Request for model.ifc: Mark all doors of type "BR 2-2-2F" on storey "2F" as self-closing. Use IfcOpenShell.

First a look at what the model holds.

```python
import ifcopenshell
import ifcopenshell.util.element

model = ifcopenshell.open("model.ifc")
print(model.schema)
storey = next(s for s in model.by_type("IfcBuildingStorey") if s.Name == "2F")
doors = [e for e in ifcopenshell.util.element.get_decomposition(storey) if e.is_a("IfcDoor")]
seen = {}
for e in doors:
    element_type = ifcopenshell.util.element.get_type(e)
    key = (element_type.Name if element_type != e and element_type else None, ifcopenshell.util.element.get_pset(e, "Pset_DoorCommon", "SelfClosing"))
    seen[key] = seen.get(key, 0) + 1
for (name, value), count in sorted(seen.items(), key=str):
    print(count, "x", name, "|", value)
```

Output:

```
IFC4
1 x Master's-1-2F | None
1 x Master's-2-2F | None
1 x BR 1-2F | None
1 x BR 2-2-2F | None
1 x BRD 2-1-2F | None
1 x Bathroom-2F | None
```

```python
import ifcopenshell
import ifcopenshell.api.pset
import ifcopenshell.util.element

model = ifcopenshell.open("model.ifc")

storey = next(s for s in model.by_type("IfcBuildingStorey") if s.Name == "2F")
doors = [e for e in ifcopenshell.util.element.get_decomposition(storey) if e.is_a("IfcDoor")]

count = 0
for e in doors:
    element_type = ifcopenshell.util.element.get_type(e)
    if element_type in (None, e) or element_type.Name != "BR 2-2-2F":
        continue
    # add_pset returns the element's existing set when there is one.
    pset = ifcopenshell.api.pset.add_pset(model, product=e, name="Pset_DoorCommon")
    ifcopenshell.api.pset.edit_pset(model, pset=pset, properties={"SelfClosing": True})
    count += 1

print(count, "doors updated")

model.write("model_updated.ifc")
```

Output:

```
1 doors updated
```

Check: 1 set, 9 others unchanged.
